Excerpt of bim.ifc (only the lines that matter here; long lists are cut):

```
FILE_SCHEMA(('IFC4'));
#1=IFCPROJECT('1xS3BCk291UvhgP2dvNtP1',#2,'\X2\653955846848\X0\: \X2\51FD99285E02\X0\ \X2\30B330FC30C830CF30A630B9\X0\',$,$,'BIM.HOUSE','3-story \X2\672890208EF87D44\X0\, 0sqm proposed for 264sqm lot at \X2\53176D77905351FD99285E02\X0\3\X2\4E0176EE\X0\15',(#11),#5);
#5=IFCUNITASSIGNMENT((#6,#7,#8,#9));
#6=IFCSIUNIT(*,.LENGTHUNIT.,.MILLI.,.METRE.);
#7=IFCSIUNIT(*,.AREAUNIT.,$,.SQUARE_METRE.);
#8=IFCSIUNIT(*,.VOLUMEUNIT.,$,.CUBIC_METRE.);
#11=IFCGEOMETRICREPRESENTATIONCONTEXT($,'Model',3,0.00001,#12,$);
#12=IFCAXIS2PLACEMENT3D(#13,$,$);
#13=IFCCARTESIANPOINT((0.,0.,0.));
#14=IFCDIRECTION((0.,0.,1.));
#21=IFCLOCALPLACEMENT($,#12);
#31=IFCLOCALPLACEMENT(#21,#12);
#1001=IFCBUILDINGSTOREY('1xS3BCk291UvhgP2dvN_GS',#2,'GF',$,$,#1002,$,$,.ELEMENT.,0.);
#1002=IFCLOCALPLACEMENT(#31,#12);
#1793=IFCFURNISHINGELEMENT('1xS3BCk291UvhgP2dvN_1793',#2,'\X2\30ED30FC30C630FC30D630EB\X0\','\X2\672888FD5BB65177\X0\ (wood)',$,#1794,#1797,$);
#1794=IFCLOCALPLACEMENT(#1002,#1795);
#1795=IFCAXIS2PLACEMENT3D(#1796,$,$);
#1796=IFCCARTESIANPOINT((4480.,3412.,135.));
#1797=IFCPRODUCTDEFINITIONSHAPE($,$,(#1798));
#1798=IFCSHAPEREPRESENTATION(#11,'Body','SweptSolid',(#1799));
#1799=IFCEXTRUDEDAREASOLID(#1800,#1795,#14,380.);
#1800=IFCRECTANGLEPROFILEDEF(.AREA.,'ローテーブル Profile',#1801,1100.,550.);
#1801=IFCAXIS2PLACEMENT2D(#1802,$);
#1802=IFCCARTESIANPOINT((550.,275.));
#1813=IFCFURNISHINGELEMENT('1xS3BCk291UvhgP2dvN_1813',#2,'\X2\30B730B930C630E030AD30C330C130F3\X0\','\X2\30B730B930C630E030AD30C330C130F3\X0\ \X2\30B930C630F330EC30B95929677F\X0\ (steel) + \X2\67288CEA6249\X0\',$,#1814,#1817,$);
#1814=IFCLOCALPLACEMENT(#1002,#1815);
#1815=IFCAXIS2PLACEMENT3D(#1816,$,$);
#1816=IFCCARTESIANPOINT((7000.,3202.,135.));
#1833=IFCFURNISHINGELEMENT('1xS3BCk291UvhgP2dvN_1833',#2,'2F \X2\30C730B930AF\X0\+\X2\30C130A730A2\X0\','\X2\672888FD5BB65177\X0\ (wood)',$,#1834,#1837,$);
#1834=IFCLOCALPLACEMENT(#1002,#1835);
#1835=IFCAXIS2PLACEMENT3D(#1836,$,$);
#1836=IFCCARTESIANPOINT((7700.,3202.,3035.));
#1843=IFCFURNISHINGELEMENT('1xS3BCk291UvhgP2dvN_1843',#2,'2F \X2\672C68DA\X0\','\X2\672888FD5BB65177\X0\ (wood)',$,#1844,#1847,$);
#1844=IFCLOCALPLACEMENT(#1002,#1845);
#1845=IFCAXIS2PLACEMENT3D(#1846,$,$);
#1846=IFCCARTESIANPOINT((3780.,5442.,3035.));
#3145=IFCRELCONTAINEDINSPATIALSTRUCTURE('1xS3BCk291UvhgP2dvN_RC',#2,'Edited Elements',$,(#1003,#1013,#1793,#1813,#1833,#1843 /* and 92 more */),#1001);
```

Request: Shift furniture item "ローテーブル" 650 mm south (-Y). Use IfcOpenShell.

```python
import ifcopenshell
import ifcopenshell.api.geometry
import ifcopenshell.util.placement
import ifcopenshell.util.unit

model = ifcopenshell.open("bim.ifc")
unit_scale = ifcopenshell.util.unit.calculate_unit_scale(model)

item = model.by_id(1793)
matrix = ifcopenshell.util.placement.get_local_placement(item.ObjectPlacement)
matrix[1, 3] -= 0.65 / unit_scale
ifcopenshell.api.geometry.edit_object_placement(model, product=item, matrix=matrix, is_si=False)

print(ifcopenshell.util.placement.get_local_placement(item.ObjectPlacement).round(3) + 0.0)

model.write("bim_v2.ifc")
```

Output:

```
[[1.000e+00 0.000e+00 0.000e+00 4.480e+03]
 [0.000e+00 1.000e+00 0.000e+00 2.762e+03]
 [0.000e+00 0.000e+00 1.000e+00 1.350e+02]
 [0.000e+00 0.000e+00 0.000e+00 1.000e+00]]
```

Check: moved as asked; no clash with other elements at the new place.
